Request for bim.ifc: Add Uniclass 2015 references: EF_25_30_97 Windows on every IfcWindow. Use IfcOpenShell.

First a look at what the model holds.

```python
import ifcopenshell

model = ifcopenshell.open("bim.ifc")
print(model.schema)
print("classifications:", [c.Name for c in model.by_type("IfcClassification")])
for ifc_class in ("IfcDoor", "IfcRoof", "IfcStair", "IfcWall", "IfcWindow"):
    print(ifc_class, len(model.by_type(ifc_class)))
```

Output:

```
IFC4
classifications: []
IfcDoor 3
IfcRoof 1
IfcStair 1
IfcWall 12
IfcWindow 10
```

```python
import ifcopenshell
import ifcopenshell.api.classification

model = ifcopenshell.open("bim.ifc")

system = ifcopenshell.api.classification.add_classification(model, classification="Uniclass 2015")

codes = {
    "IfcWindow": ("EF_25_30_97", "Windows"),
}
for ifc_class, (code, name) in codes.items():
    products = model.by_type(ifc_class)
    ifcopenshell.api.classification.add_reference(
        model, products=products, classification=system, identification=code, name=name
    )
    print(code, len(products))

model.write("bim_rev.ifc")
```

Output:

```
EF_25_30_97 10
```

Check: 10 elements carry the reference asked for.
